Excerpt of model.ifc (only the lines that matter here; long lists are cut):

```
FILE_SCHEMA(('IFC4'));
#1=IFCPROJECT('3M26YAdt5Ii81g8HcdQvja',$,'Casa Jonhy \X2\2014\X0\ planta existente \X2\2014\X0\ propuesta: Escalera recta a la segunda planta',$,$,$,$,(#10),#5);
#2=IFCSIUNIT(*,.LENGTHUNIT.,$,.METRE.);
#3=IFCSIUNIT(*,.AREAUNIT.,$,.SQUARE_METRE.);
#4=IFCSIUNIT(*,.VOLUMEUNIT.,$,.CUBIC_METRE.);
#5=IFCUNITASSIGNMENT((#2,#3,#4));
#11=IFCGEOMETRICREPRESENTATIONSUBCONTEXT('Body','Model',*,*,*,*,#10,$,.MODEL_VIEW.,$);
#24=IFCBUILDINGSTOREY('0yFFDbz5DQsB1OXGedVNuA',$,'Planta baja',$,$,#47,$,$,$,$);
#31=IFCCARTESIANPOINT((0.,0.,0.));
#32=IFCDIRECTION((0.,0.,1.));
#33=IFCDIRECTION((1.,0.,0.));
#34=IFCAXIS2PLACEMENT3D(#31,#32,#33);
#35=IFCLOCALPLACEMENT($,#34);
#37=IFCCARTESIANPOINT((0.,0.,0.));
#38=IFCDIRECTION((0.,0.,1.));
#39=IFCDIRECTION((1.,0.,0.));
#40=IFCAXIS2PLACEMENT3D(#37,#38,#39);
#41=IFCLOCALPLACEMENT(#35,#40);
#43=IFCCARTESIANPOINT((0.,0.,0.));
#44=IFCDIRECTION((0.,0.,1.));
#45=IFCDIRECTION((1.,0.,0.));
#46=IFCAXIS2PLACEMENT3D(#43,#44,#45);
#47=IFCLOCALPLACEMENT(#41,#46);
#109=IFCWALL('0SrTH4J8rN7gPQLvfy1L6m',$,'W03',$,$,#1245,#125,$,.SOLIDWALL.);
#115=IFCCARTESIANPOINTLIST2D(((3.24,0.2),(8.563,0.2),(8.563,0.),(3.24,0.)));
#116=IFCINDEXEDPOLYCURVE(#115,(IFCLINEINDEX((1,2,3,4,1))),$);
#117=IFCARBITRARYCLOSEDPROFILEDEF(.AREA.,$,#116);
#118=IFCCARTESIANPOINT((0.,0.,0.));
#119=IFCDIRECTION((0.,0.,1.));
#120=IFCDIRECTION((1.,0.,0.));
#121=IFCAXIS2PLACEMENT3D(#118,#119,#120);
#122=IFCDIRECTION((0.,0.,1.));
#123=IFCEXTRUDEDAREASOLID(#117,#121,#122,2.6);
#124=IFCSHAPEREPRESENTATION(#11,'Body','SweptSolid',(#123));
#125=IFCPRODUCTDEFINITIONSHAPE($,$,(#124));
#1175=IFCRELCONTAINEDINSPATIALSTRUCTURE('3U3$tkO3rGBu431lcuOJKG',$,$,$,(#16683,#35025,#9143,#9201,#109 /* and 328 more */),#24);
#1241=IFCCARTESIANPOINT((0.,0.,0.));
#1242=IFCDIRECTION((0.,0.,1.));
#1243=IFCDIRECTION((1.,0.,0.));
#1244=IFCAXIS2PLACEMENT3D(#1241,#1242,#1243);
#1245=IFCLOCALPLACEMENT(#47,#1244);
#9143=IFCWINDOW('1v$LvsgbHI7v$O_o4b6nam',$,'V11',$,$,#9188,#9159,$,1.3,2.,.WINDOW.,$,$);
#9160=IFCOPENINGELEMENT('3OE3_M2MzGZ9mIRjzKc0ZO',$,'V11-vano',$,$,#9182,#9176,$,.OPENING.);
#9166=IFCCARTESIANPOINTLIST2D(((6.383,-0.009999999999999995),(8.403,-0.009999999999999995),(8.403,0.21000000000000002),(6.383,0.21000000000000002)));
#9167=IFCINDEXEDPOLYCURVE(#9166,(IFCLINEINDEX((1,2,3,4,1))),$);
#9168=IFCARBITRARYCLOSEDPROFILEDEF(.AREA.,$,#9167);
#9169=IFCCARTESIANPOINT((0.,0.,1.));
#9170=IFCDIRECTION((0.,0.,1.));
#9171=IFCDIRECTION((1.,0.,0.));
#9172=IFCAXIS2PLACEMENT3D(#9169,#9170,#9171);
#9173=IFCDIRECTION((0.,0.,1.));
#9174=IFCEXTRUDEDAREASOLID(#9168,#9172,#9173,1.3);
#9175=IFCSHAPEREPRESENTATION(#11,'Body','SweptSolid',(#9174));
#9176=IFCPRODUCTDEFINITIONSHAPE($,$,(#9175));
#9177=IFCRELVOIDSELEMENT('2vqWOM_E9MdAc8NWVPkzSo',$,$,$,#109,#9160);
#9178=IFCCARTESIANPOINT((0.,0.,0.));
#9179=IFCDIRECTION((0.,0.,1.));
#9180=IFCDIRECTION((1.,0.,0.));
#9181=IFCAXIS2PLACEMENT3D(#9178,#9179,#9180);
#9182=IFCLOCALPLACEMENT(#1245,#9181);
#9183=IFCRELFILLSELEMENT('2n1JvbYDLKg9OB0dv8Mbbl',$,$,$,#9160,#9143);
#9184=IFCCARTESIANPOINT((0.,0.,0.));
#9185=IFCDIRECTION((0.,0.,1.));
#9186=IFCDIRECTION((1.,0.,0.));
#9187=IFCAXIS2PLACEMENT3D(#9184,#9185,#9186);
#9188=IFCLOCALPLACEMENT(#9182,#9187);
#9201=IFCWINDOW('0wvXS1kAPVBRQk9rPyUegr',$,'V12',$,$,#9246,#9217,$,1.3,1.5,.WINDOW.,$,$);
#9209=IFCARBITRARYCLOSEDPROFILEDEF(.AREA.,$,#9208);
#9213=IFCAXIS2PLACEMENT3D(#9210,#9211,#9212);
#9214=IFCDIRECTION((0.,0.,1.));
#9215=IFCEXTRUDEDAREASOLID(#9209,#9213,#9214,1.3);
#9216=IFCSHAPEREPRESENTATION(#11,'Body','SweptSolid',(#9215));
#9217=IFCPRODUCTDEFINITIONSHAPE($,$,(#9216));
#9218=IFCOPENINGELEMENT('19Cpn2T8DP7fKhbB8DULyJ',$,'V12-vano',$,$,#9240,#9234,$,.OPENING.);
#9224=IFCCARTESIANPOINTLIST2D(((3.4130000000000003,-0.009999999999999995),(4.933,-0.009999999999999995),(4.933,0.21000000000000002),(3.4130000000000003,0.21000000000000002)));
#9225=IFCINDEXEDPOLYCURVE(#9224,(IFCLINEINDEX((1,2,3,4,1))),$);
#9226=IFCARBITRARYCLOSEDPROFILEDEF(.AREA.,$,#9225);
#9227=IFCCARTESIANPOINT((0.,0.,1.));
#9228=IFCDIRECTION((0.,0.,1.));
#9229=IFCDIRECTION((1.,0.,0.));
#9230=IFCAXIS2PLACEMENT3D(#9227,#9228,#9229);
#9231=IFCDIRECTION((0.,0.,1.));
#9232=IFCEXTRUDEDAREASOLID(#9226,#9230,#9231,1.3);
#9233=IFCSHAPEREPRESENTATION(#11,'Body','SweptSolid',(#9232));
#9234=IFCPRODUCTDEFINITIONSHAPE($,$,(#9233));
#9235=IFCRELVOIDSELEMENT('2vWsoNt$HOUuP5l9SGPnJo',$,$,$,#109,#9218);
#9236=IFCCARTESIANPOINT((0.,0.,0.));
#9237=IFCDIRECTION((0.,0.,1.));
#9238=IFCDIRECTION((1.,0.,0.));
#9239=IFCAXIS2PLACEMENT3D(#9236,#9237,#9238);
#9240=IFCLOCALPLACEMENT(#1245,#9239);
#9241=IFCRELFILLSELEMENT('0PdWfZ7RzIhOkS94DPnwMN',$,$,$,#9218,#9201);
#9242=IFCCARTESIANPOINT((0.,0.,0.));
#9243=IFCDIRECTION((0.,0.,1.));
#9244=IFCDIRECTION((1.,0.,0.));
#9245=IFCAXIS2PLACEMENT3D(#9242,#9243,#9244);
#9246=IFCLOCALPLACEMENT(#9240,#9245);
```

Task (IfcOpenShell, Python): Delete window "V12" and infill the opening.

```python
import ifcopenshell
import ifcopenshell.api.feature
import ifcopenshell.api.root
import ifcopenshell.geom
import ifcopenshell.util.shape

model = ifcopenshell.open("model.ifc")
settings = ifcopenshell.geom.settings()


def volume(element):
    """Net volume in cubic metres, openings subtracted."""
    shape = ifcopenshell.geom.create_shape(settings, element)
    return ifcopenshell.util.shape.get_volume(shape.geometry)


window = model.by_guid("0wvXS1kAPVBRQk9rPyUegr")
opening = window.FillsVoids[0].RelatingOpeningElement
wall = opening.VoidsElements[0].RelatingBuildingElement
before = volume(wall)

ifcopenshell.api.root.remove_product(model, product=window)
ifcopenshell.api.feature.remove_feature(model, feature=opening)

after = volume(wall)

print(f"wall volume {before:.3f} -> {after:.3f} m3")

model.write("model_v2.ifc")
```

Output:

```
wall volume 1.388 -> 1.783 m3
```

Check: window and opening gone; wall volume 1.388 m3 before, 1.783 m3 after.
